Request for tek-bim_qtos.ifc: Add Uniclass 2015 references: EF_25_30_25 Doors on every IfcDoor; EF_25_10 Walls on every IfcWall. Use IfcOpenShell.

First a look at what the model holds.

```python
import ifcopenshell

model = ifcopenshell.open("tek-bim_qtos.ifc")
print(model.schema)
print("classifications:", [c.Name for c in model.by_type("IfcClassification")])
for ifc_class in ("IfcDoor", "IfcRoof", "IfcStair", "IfcWall", "IfcWindow"):
    print(ifc_class, len(model.by_type(ifc_class)))
```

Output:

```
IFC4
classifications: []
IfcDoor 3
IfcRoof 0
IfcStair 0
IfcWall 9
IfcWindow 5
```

```python
import ifcopenshell
import ifcopenshell.api.classification

model = ifcopenshell.open("tek-bim_qtos.ifc")

system = ifcopenshell.api.classification.add_classification(model, classification="Uniclass 2015")

codes = {
    "IfcDoor": ("EF_25_30_25", "Doors"),
    "IfcWall": ("EF_25_10", "Walls"),
}
for ifc_class, (code, name) in codes.items():
    products = model.by_type(ifc_class)
    ifcopenshell.api.classification.add_reference(
        model, products=products, classification=system, identification=code, name=name
    )
    print(code, len(products))

model.write("tek-bim_qtos_rev.ifc")
```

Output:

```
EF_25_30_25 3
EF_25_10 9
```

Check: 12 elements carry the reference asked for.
